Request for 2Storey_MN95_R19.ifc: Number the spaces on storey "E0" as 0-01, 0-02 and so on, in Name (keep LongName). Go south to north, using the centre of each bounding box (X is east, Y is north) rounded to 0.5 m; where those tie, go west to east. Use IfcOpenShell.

First a look at what the model holds.

```python
import ifcopenshell
import ifcopenshell.util.element
import ifcopenshell.util.placement

model = ifcopenshell.open("2Storey_MN95_R19.ifc")
print(model.schema)
storey = next(s for s in model.by_type("IfcBuildingStorey") if s.Name == "E0")
spaces = [e for e in ifcopenshell.util.element.get_decomposition(storey) if e.is_a("IfcSpace")]
for e in sorted(spaces, key=lambda e: e.id()):
    origin = ifcopenshell.util.placement.get_local_placement(e.ObjectPlacement)[:3, 3]
    print(e.id(), e.Name, e.LongName, origin.round(2) + 0.0, sep=" | ")
```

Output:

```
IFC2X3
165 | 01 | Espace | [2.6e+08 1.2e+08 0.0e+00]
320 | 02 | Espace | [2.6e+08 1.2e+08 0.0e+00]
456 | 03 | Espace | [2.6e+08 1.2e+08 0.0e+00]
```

```python
import ifcopenshell
import ifcopenshell.geom
import ifcopenshell.util.element
import ifcopenshell.util.shape

model = ifcopenshell.open("2Storey_MN95_R19.ifc")
settings = ifcopenshell.geom.settings()
settings.set("use-world-coords", True)


def centre(element):
    shape = ifcopenshell.geom.create_shape(settings, element)
    return ifcopenshell.util.shape.get_bbox_centroid(shape.geometry)


storey = next(s for s in model.by_type("IfcBuildingStorey") if s.Name == "E0")
spaces = [e for e in ifcopenshell.util.element.get_decomposition(storey) if e.is_a("IfcSpace")]

# Insertion points can sit at a corner or the storey origin, so sort by the geometry (in metres).
centres = {e: centre(e) for e in spaces}
spaces.sort(key=lambda e: (round(centres[e][1] / 0.5), centres[e][0]))

for i, e in enumerate(spaces, start=1):
    number = f"0-{i:02d}"
    e.Name = number
    print(e.id(), number)

model.write("2Storey_MN95_R19_updated.ifc")
```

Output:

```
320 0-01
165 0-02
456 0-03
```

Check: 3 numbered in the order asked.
